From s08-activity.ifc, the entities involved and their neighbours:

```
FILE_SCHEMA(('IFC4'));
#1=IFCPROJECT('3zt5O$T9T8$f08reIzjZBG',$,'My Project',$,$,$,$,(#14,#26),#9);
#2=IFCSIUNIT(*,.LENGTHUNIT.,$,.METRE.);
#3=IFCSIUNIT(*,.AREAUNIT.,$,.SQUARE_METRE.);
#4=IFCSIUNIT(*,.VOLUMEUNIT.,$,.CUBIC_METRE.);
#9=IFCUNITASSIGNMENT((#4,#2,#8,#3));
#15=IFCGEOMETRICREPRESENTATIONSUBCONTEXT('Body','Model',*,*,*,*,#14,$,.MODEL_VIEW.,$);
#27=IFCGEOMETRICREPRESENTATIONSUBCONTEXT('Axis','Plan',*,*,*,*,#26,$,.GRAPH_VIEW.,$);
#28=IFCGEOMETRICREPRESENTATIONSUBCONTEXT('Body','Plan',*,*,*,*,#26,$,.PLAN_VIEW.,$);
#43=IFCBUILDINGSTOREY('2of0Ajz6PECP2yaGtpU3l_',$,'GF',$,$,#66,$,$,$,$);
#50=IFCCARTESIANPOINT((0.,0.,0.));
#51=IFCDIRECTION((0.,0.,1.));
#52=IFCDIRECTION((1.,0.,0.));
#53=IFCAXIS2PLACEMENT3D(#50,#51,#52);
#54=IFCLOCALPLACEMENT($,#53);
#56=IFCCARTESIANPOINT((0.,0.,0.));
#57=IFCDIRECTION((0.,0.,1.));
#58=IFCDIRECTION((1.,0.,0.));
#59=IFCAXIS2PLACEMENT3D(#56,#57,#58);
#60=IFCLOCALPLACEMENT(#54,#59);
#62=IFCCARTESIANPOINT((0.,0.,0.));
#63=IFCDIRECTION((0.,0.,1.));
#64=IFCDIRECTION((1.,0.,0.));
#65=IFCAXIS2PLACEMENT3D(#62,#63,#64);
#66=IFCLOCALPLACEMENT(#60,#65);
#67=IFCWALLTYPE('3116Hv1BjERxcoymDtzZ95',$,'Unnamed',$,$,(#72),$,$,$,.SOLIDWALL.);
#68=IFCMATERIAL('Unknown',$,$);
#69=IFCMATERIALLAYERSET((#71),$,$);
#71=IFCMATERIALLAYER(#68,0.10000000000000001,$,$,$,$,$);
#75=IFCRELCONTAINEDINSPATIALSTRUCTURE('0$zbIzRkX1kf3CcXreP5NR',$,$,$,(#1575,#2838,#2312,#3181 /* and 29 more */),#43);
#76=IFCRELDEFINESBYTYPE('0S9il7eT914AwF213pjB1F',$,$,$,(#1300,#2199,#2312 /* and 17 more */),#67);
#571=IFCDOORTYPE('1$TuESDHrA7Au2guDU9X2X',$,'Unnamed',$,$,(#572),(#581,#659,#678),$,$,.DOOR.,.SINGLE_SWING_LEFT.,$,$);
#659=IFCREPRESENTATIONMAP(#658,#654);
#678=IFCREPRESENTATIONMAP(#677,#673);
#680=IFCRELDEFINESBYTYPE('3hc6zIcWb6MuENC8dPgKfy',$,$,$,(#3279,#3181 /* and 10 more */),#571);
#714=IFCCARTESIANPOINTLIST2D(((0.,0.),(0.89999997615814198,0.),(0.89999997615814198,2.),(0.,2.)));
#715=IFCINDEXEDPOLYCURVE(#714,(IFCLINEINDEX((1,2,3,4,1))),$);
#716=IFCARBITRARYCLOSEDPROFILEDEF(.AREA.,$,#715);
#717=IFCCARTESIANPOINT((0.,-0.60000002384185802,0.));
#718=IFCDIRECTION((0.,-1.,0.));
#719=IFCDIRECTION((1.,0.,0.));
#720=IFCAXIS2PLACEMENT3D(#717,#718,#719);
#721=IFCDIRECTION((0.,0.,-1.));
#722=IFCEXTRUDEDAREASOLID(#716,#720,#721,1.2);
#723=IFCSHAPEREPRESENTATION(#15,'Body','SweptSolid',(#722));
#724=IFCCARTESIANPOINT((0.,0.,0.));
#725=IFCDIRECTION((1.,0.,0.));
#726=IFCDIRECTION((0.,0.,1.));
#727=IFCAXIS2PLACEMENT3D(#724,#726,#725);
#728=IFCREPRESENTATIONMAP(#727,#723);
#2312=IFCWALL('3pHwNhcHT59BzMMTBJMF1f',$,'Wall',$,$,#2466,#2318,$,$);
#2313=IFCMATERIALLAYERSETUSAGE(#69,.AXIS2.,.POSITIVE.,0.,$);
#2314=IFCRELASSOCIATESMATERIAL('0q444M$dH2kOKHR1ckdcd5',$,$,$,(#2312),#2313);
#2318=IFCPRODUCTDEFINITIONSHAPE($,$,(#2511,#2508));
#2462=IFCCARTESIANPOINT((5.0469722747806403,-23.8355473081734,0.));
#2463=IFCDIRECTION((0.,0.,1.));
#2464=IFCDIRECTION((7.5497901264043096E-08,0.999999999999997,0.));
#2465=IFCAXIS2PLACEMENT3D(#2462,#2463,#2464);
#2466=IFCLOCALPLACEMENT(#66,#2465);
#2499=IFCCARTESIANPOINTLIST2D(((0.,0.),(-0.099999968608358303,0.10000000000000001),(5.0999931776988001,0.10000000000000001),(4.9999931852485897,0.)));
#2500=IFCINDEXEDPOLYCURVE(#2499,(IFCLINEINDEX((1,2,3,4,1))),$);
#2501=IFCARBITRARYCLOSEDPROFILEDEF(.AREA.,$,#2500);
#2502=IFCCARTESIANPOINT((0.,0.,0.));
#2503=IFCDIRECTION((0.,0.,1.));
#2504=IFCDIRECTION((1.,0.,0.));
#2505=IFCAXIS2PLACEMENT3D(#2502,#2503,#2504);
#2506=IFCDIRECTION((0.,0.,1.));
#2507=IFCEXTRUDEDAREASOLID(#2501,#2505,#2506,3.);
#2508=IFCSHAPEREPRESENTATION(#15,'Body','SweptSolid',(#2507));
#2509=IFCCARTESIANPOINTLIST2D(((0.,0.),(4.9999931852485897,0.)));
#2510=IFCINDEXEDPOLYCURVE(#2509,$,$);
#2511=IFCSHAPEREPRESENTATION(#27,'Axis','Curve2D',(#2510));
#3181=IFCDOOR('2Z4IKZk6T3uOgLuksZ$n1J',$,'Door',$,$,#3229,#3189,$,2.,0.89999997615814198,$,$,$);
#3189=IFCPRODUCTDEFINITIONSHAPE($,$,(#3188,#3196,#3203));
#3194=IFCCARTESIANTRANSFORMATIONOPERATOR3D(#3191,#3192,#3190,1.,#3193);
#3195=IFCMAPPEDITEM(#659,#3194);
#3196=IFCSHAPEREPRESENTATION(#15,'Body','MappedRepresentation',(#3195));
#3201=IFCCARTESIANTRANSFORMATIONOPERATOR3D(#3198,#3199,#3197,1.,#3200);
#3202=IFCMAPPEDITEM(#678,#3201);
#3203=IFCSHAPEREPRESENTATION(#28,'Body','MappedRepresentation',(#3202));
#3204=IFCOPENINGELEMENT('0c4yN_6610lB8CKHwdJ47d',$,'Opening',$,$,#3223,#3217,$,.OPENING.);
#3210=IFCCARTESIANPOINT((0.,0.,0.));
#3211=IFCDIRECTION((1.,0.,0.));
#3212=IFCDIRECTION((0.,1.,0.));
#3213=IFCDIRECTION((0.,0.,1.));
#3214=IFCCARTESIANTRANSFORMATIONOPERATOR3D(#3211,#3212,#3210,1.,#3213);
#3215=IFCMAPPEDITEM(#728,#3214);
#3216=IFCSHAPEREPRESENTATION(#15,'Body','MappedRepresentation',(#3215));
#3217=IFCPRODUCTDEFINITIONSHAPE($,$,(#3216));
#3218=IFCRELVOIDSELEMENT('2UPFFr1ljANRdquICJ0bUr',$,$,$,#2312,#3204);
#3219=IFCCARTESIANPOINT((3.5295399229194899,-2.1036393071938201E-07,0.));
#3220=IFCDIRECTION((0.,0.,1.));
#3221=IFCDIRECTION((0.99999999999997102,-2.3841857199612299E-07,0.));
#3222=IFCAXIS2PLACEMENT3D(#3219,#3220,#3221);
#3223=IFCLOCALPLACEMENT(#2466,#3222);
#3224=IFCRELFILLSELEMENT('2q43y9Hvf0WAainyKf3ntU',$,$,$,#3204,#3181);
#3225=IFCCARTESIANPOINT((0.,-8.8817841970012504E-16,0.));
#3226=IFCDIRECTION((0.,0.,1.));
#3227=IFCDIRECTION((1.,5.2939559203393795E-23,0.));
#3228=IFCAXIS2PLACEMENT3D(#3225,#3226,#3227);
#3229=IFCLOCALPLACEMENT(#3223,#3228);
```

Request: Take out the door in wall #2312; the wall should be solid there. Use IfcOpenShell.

```python
import ifcopenshell
import ifcopenshell.api.feature
import ifcopenshell.api.root
import ifcopenshell.geom
import ifcopenshell.util.shape

model = ifcopenshell.open("s08-activity.ifc")
settings = ifcopenshell.geom.settings()


def volume(element):
    """Net volume in cubic metres, openings subtracted."""
    shape = ifcopenshell.geom.create_shape(settings, element)
    return ifcopenshell.util.shape.get_volume(shape.geometry)


door = model.by_id(3181)
opening = door.FillsVoids[0].RelatingOpeningElement
wall = opening.VoidsElements[0].RelatingBuildingElement
before = volume(wall)

ifcopenshell.api.root.remove_product(model, product=door)
ifcopenshell.api.feature.remove_feature(model, feature=opening)

after = volume(wall)

print(f"wall volume {before:.3f} -> {after:.3f} m3")

model.write("s08-activity-out.ifc")
```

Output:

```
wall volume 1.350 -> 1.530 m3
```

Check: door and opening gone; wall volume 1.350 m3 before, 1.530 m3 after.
